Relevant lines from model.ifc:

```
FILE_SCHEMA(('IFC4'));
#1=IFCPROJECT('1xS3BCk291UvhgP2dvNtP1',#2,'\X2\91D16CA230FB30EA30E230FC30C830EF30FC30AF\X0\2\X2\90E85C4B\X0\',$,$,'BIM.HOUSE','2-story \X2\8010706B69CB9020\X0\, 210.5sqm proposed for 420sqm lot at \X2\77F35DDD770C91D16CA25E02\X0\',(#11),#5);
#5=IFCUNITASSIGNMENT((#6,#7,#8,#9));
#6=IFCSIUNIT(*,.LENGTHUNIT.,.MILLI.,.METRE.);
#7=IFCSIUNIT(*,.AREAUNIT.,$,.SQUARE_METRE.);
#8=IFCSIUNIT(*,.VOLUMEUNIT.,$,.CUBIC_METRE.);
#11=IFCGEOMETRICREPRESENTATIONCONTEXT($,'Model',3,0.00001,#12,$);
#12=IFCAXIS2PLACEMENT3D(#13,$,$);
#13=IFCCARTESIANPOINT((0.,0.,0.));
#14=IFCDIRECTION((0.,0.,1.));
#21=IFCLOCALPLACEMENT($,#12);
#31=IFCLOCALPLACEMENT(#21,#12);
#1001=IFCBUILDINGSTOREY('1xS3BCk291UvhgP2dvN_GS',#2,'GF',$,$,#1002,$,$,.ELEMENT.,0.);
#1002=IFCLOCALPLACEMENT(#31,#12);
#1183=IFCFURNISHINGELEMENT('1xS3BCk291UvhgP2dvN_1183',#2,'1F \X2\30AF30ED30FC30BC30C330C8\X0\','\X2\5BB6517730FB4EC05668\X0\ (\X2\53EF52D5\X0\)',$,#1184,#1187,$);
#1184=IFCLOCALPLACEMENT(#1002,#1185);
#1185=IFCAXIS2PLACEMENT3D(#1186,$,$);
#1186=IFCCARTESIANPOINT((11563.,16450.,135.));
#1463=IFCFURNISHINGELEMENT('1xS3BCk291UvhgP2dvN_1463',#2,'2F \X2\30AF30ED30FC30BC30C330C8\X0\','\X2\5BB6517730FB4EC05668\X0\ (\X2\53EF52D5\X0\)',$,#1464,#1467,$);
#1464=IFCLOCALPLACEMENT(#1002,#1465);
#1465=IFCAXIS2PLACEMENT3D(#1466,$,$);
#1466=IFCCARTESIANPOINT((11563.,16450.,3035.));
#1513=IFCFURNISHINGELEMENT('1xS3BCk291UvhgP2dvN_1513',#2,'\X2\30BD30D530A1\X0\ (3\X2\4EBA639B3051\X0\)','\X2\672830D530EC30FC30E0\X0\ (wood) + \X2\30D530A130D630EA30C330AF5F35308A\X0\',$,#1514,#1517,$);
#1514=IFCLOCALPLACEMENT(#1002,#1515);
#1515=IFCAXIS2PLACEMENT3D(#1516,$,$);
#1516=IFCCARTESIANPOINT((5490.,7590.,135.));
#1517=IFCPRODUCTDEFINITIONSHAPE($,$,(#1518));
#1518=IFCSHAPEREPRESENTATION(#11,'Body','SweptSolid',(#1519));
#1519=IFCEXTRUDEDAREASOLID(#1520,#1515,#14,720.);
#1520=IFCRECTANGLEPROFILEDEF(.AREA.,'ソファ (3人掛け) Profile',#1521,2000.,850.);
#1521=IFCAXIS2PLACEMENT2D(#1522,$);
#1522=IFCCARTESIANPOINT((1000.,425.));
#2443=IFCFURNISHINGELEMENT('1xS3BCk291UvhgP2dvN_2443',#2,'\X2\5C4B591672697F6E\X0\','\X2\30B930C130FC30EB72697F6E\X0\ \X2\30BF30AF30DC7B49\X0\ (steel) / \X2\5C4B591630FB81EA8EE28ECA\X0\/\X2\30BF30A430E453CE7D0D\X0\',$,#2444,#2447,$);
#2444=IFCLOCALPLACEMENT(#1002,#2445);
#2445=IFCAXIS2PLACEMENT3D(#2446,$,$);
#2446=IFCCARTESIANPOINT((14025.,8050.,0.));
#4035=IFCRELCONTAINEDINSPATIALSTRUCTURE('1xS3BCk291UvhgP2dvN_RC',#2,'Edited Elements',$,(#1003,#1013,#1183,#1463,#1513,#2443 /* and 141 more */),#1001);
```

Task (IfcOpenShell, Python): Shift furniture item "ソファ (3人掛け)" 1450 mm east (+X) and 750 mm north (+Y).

```python
import ifcopenshell
import ifcopenshell.api.geometry
import ifcopenshell.util.placement
import ifcopenshell.util.unit

model = ifcopenshell.open("model.ifc")
unit_scale = ifcopenshell.util.unit.calculate_unit_scale(model)

item = model.by_guid("1xS3BCk291UvhgP2dvN_1513")
matrix = ifcopenshell.util.placement.get_local_placement(item.ObjectPlacement)
matrix[0, 3] += 1.45 / unit_scale
matrix[1, 3] += 0.75 / unit_scale
ifcopenshell.api.geometry.edit_object_placement(model, product=item, matrix=matrix, is_si=False)

print(ifcopenshell.util.placement.get_local_placement(item.ObjectPlacement).round(3) + 0.0)

model.write("model_updated.ifc")
```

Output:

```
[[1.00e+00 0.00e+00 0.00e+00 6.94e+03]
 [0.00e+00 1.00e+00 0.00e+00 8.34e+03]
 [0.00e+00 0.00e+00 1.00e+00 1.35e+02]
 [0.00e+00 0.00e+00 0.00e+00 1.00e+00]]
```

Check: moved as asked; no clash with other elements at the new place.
